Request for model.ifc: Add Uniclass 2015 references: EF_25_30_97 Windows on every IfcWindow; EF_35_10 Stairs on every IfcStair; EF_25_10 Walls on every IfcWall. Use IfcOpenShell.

First a look at what the model holds.

```python
import ifcopenshell

model = ifcopenshell.open("model.ifc")
print(model.schema)
print("classifications:", [c.Name for c in model.by_type("IfcClassification")])
for ifc_class in ("IfcDoor", "IfcRoof", "IfcStair", "IfcWall", "IfcWindow"):
    print(ifc_class, len(model.by_type(ifc_class)))
```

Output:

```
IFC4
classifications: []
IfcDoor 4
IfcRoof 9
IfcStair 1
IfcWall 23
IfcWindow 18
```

```python
import ifcopenshell
import ifcopenshell.api.classification

model = ifcopenshell.open("model.ifc")

system = ifcopenshell.api.classification.add_classification(model, classification="Uniclass 2015")

codes = {
    "IfcWindow": ("EF_25_30_97", "Windows"),
    "IfcStair": ("EF_35_10", "Stairs"),
    "IfcWall": ("EF_25_10", "Walls"),
}
for ifc_class, (code, name) in codes.items():
    products = model.by_type(ifc_class)
    ifcopenshell.api.classification.add_reference(
        model, products=products, classification=system, identification=code, name=name
    )
    print(code, len(products))

model.write("model_v2.ifc")
```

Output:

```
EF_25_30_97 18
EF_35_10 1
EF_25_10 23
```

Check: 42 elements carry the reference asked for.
